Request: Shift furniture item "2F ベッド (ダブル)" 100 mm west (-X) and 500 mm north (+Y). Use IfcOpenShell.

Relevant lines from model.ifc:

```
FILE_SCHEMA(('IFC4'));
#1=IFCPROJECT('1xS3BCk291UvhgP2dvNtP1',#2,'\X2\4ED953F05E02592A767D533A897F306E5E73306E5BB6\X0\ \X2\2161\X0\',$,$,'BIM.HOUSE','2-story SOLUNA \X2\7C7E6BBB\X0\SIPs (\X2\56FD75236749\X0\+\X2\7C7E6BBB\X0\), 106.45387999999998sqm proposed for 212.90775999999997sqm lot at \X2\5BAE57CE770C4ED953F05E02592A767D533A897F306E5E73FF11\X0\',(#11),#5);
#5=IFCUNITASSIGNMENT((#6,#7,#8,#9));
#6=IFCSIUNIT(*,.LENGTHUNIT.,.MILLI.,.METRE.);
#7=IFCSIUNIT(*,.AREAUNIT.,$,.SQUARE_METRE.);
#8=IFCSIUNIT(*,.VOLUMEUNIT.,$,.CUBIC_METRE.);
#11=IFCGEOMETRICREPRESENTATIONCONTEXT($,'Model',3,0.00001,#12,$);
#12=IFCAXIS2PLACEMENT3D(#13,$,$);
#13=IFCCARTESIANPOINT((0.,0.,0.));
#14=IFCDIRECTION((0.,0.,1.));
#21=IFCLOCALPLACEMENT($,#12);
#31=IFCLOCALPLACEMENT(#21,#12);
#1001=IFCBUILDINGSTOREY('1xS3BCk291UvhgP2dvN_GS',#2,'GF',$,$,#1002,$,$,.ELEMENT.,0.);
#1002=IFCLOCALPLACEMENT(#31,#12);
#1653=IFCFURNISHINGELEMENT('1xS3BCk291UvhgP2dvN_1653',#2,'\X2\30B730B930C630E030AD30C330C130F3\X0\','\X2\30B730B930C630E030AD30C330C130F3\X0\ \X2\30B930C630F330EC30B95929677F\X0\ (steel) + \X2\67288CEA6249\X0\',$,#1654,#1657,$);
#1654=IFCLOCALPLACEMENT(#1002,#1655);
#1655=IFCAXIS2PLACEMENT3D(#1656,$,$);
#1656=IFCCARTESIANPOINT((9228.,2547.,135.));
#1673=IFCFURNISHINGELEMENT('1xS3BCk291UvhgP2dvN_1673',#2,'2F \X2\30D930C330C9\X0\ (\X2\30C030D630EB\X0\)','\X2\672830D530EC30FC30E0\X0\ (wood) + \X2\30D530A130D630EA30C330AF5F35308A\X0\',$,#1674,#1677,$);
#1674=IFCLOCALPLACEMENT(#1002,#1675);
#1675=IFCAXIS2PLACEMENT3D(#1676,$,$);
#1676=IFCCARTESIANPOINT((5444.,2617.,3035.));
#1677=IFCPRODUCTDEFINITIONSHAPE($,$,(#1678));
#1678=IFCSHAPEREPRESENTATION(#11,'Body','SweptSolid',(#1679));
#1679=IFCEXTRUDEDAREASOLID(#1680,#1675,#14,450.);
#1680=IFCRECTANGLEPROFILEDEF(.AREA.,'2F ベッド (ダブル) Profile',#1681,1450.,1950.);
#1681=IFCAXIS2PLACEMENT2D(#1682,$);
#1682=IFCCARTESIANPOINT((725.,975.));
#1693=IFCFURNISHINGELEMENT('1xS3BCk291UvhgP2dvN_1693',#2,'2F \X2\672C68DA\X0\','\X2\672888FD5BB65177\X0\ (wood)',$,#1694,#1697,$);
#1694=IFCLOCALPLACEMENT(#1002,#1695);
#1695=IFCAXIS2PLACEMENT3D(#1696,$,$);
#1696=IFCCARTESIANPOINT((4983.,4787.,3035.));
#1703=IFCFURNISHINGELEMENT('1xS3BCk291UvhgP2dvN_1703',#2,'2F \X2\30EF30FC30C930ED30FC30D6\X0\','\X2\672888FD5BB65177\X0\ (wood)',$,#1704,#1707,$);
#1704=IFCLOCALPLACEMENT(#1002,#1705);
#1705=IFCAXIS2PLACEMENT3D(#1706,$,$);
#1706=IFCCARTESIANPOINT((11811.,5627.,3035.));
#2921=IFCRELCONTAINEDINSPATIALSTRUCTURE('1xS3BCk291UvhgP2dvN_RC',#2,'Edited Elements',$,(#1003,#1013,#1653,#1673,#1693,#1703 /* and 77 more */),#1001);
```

```python
import ifcopenshell
import ifcopenshell.api.geometry
import ifcopenshell.util.placement
import ifcopenshell.util.unit

model = ifcopenshell.open("model.ifc")
unit_scale = ifcopenshell.util.unit.calculate_unit_scale(model)

item = model.by_id(1673)
matrix = ifcopenshell.util.placement.get_local_placement(item.ObjectPlacement)
matrix[0, 3] -= 0.1 / unit_scale
matrix[1, 3] += 0.5 / unit_scale
ifcopenshell.api.geometry.edit_object_placement(model, product=item, matrix=matrix, is_si=False)

print(ifcopenshell.util.placement.get_local_placement(item.ObjectPlacement).round(3) + 0.0)

model.write("model_edited.ifc")
```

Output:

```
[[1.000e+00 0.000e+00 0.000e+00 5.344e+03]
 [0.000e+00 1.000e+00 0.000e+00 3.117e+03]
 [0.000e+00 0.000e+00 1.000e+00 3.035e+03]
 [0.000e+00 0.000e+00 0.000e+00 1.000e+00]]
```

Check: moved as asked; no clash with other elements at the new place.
